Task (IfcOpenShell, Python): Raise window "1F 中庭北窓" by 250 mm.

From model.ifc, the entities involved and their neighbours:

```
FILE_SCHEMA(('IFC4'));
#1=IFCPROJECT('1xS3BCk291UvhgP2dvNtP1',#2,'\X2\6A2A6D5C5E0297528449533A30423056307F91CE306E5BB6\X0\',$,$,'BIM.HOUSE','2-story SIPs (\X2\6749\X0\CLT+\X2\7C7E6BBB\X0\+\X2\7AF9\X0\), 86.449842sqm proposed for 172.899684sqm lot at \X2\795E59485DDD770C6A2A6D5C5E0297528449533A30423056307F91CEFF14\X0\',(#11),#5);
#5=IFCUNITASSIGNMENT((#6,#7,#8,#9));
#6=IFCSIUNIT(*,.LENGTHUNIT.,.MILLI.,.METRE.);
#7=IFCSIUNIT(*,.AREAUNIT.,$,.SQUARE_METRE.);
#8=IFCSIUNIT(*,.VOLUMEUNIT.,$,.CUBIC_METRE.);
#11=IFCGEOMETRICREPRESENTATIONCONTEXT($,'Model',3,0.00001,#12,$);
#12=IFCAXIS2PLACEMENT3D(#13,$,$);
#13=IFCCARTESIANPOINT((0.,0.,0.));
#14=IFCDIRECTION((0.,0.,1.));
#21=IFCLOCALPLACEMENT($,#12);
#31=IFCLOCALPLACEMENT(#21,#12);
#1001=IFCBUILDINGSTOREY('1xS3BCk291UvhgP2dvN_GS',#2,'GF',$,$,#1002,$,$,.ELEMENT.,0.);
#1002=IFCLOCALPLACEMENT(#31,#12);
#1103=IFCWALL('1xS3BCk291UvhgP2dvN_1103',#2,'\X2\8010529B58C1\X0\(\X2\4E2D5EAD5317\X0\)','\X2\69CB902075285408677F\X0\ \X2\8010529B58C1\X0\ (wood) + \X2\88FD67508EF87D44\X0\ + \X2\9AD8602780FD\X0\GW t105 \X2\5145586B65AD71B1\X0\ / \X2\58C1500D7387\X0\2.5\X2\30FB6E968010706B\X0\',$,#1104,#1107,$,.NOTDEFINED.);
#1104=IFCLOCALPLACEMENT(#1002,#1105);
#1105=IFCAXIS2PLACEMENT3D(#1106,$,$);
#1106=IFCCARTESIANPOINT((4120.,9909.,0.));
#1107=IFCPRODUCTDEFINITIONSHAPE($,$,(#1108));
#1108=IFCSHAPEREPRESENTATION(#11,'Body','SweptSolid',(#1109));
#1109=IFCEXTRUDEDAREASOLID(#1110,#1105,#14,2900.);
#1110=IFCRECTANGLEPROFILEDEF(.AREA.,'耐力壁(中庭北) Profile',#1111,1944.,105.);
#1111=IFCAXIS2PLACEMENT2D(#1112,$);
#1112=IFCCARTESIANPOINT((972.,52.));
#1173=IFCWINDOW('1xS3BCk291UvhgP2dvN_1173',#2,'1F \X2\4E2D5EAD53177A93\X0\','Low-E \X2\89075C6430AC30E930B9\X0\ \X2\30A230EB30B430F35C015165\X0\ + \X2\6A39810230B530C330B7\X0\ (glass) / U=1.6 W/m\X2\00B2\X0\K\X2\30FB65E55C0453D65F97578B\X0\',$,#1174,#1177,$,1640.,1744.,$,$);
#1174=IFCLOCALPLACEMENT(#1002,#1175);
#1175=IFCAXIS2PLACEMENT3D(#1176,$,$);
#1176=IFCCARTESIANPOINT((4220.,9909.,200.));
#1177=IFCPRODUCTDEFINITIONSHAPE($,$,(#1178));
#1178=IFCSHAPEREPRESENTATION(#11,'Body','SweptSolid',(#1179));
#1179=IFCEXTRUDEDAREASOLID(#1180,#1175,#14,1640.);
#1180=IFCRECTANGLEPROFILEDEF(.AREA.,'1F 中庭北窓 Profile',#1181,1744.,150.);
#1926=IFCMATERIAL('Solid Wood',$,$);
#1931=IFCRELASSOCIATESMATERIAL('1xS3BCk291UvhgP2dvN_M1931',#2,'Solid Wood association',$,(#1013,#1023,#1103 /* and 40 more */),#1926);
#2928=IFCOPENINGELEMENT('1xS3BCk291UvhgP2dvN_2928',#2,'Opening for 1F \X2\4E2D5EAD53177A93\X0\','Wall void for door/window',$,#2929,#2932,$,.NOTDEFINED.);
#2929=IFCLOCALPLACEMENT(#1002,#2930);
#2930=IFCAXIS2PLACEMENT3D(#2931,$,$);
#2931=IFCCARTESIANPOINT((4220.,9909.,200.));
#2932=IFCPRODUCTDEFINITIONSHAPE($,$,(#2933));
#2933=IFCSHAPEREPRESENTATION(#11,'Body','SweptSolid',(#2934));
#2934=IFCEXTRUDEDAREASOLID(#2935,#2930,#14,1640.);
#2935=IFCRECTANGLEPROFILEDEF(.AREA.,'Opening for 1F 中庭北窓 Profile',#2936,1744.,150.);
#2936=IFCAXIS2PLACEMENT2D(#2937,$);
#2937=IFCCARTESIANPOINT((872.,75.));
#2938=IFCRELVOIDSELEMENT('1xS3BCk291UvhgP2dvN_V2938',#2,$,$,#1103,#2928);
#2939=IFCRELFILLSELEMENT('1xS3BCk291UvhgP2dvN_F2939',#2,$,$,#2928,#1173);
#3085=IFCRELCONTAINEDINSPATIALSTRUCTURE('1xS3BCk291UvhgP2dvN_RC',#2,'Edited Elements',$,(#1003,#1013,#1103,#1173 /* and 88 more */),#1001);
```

```python
import numpy as np
import ifcopenshell
import ifcopenshell.api.geometry
import ifcopenshell.util.placement
import ifcopenshell.util.unit

model = ifcopenshell.open("model.ifc")
unit_scale = ifcopenshell.util.unit.calculate_unit_scale(model)

window = model.by_guid("1xS3BCk291UvhgP2dvN_1173")
opening = window.FillsVoids[0].RelatingOpeningElement
dz = 250.0

shift = np.array([0.0, 0.0, dz])
# The window is not placed relative to its opening, so move both.
for product in (opening, window):
    matrix = ifcopenshell.util.placement.get_local_placement(product.ObjectPlacement)
    matrix[:3, 3] += shift
    ifcopenshell.api.geometry.edit_object_placement(model, product=product, matrix=matrix, is_si=False)

print(f"moved by {dz * unit_scale:+.3f} m")

model.write("model_v2.ifc")
```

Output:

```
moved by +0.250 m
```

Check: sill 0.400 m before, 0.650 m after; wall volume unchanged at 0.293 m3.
